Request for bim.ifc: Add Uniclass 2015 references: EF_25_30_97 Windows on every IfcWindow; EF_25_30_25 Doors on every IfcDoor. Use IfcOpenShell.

First a look at what the model holds.

```python
import ifcopenshell

model = ifcopenshell.open("bim.ifc")
print(model.schema)
print("classifications:", [c.Name for c in model.by_type("IfcClassification")])
for ifc_class in ("IfcDoor", "IfcRoof", "IfcStair", "IfcWall", "IfcWindow"):
    print(ifc_class, len(model.by_type(ifc_class)))
```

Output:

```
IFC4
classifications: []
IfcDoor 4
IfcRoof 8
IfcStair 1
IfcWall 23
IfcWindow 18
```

```python
import ifcopenshell
import ifcopenshell.api.classification

model = ifcopenshell.open("bim.ifc")

system = ifcopenshell.api.classification.add_classification(model, classification="Uniclass 2015")

codes = {
    "IfcWindow": ("EF_25_30_97", "Windows"),
    "IfcDoor": ("EF_25_30_25", "Doors"),
}
for ifc_class, (code, name) in codes.items():
    products = model.by_type(ifc_class)
    ifcopenshell.api.classification.add_reference(
        model, products=products, classification=system, identification=code, name=name
    )
    print(code, len(products))

model.write("bim_edited.ifc")
```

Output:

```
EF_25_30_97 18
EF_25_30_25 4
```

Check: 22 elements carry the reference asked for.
